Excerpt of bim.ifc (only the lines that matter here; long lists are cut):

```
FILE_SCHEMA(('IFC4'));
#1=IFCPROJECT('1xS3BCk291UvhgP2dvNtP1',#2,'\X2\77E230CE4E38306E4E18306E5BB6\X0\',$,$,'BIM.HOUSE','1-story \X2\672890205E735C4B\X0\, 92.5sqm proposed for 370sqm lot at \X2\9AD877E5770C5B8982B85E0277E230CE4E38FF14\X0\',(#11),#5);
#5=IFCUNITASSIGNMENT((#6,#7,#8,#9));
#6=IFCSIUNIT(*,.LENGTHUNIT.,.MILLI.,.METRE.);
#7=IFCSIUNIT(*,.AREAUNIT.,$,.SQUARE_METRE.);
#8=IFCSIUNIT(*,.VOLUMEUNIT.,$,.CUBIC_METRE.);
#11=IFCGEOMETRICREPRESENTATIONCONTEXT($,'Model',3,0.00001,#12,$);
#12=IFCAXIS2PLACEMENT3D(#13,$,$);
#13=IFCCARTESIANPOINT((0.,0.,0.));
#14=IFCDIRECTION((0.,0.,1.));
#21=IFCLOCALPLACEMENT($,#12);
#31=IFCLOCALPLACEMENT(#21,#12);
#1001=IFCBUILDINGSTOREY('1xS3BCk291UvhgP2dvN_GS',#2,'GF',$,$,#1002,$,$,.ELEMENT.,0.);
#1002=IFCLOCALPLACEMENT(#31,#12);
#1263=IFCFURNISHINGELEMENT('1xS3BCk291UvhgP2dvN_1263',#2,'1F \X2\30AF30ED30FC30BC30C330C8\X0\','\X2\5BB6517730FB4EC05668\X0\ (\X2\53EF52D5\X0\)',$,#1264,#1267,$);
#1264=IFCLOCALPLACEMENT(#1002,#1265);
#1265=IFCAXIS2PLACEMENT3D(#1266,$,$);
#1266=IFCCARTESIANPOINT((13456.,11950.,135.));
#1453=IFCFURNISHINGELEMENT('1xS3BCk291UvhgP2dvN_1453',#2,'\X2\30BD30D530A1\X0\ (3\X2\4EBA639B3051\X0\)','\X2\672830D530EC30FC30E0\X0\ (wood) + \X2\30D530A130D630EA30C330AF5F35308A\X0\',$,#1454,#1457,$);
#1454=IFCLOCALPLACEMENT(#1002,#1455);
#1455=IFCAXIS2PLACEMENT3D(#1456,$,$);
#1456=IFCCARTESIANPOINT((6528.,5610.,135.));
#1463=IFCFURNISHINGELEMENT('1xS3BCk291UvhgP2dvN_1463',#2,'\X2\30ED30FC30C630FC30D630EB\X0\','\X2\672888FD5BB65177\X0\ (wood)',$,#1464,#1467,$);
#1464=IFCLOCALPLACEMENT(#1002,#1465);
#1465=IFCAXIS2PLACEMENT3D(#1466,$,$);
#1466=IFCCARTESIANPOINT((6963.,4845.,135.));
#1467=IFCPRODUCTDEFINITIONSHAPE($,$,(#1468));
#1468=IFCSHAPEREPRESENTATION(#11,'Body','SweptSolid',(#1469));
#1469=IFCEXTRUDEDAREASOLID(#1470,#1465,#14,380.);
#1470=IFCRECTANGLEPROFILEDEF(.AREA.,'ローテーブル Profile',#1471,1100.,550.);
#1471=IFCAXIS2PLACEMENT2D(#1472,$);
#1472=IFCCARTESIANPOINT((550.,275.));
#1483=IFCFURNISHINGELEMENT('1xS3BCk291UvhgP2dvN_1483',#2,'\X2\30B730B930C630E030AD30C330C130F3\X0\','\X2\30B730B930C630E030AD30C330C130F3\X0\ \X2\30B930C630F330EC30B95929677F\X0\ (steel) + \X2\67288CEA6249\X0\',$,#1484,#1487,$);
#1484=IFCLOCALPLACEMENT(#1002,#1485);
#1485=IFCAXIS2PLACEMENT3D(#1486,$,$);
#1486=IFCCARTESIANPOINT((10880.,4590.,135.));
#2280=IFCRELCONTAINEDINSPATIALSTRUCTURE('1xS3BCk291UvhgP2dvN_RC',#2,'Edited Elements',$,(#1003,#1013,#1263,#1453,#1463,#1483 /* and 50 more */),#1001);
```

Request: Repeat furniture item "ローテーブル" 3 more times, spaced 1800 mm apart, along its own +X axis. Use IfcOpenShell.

```python
import ifcopenshell
import ifcopenshell.api.geometry
import ifcopenshell.api.root
import ifcopenshell.util.element
import ifcopenshell.util.placement
import ifcopenshell.util.unit

model = ifcopenshell.open("bim.ifc")
unit_scale = ifcopenshell.util.unit.calculate_unit_scale(model)


def reuse_history(source, copy):
    """copy_class also copies each property set's owner history, people and application; keep the originals."""
    for rel in copy.IsDefinedBy:
        if rel.is_a("IfcRelDefinesByProperties") and (history := rel.RelatingPropertyDefinition.OwnerHistory):
            rel.RelatingPropertyDefinition.OwnerHistory = source.OwnerHistory
            ifcopenshell.util.element.remove_deep2(model, history)


source = model.by_guid("1xS3BCk291UvhgP2dvN_1463")
base = ifcopenshell.util.placement.get_local_placement(source.ObjectPlacement)
step = base[:3, 0] * 1.8 / unit_scale

for i in range(1, 4):
    copy = ifcopenshell.api.root.copy_class(model, product=source)
    copy.Representation = ifcopenshell.util.element.copy_deep(
        model, source.Representation, exclude=["IfcGeometricRepresentationContext", "IfcRepresentationMap"]
    )
    reuse_history(source, copy)
    matrix = base.copy()
    matrix[:3, 3] += i * step
    print("added at", matrix[:3, 3].round(3) + 0.0)
    ifcopenshell.api.geometry.edit_object_placement(model, product=copy, matrix=matrix, is_si=False)

model.write("bim_edited.ifc")
```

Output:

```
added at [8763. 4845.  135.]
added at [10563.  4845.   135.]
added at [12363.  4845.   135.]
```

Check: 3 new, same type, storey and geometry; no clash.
